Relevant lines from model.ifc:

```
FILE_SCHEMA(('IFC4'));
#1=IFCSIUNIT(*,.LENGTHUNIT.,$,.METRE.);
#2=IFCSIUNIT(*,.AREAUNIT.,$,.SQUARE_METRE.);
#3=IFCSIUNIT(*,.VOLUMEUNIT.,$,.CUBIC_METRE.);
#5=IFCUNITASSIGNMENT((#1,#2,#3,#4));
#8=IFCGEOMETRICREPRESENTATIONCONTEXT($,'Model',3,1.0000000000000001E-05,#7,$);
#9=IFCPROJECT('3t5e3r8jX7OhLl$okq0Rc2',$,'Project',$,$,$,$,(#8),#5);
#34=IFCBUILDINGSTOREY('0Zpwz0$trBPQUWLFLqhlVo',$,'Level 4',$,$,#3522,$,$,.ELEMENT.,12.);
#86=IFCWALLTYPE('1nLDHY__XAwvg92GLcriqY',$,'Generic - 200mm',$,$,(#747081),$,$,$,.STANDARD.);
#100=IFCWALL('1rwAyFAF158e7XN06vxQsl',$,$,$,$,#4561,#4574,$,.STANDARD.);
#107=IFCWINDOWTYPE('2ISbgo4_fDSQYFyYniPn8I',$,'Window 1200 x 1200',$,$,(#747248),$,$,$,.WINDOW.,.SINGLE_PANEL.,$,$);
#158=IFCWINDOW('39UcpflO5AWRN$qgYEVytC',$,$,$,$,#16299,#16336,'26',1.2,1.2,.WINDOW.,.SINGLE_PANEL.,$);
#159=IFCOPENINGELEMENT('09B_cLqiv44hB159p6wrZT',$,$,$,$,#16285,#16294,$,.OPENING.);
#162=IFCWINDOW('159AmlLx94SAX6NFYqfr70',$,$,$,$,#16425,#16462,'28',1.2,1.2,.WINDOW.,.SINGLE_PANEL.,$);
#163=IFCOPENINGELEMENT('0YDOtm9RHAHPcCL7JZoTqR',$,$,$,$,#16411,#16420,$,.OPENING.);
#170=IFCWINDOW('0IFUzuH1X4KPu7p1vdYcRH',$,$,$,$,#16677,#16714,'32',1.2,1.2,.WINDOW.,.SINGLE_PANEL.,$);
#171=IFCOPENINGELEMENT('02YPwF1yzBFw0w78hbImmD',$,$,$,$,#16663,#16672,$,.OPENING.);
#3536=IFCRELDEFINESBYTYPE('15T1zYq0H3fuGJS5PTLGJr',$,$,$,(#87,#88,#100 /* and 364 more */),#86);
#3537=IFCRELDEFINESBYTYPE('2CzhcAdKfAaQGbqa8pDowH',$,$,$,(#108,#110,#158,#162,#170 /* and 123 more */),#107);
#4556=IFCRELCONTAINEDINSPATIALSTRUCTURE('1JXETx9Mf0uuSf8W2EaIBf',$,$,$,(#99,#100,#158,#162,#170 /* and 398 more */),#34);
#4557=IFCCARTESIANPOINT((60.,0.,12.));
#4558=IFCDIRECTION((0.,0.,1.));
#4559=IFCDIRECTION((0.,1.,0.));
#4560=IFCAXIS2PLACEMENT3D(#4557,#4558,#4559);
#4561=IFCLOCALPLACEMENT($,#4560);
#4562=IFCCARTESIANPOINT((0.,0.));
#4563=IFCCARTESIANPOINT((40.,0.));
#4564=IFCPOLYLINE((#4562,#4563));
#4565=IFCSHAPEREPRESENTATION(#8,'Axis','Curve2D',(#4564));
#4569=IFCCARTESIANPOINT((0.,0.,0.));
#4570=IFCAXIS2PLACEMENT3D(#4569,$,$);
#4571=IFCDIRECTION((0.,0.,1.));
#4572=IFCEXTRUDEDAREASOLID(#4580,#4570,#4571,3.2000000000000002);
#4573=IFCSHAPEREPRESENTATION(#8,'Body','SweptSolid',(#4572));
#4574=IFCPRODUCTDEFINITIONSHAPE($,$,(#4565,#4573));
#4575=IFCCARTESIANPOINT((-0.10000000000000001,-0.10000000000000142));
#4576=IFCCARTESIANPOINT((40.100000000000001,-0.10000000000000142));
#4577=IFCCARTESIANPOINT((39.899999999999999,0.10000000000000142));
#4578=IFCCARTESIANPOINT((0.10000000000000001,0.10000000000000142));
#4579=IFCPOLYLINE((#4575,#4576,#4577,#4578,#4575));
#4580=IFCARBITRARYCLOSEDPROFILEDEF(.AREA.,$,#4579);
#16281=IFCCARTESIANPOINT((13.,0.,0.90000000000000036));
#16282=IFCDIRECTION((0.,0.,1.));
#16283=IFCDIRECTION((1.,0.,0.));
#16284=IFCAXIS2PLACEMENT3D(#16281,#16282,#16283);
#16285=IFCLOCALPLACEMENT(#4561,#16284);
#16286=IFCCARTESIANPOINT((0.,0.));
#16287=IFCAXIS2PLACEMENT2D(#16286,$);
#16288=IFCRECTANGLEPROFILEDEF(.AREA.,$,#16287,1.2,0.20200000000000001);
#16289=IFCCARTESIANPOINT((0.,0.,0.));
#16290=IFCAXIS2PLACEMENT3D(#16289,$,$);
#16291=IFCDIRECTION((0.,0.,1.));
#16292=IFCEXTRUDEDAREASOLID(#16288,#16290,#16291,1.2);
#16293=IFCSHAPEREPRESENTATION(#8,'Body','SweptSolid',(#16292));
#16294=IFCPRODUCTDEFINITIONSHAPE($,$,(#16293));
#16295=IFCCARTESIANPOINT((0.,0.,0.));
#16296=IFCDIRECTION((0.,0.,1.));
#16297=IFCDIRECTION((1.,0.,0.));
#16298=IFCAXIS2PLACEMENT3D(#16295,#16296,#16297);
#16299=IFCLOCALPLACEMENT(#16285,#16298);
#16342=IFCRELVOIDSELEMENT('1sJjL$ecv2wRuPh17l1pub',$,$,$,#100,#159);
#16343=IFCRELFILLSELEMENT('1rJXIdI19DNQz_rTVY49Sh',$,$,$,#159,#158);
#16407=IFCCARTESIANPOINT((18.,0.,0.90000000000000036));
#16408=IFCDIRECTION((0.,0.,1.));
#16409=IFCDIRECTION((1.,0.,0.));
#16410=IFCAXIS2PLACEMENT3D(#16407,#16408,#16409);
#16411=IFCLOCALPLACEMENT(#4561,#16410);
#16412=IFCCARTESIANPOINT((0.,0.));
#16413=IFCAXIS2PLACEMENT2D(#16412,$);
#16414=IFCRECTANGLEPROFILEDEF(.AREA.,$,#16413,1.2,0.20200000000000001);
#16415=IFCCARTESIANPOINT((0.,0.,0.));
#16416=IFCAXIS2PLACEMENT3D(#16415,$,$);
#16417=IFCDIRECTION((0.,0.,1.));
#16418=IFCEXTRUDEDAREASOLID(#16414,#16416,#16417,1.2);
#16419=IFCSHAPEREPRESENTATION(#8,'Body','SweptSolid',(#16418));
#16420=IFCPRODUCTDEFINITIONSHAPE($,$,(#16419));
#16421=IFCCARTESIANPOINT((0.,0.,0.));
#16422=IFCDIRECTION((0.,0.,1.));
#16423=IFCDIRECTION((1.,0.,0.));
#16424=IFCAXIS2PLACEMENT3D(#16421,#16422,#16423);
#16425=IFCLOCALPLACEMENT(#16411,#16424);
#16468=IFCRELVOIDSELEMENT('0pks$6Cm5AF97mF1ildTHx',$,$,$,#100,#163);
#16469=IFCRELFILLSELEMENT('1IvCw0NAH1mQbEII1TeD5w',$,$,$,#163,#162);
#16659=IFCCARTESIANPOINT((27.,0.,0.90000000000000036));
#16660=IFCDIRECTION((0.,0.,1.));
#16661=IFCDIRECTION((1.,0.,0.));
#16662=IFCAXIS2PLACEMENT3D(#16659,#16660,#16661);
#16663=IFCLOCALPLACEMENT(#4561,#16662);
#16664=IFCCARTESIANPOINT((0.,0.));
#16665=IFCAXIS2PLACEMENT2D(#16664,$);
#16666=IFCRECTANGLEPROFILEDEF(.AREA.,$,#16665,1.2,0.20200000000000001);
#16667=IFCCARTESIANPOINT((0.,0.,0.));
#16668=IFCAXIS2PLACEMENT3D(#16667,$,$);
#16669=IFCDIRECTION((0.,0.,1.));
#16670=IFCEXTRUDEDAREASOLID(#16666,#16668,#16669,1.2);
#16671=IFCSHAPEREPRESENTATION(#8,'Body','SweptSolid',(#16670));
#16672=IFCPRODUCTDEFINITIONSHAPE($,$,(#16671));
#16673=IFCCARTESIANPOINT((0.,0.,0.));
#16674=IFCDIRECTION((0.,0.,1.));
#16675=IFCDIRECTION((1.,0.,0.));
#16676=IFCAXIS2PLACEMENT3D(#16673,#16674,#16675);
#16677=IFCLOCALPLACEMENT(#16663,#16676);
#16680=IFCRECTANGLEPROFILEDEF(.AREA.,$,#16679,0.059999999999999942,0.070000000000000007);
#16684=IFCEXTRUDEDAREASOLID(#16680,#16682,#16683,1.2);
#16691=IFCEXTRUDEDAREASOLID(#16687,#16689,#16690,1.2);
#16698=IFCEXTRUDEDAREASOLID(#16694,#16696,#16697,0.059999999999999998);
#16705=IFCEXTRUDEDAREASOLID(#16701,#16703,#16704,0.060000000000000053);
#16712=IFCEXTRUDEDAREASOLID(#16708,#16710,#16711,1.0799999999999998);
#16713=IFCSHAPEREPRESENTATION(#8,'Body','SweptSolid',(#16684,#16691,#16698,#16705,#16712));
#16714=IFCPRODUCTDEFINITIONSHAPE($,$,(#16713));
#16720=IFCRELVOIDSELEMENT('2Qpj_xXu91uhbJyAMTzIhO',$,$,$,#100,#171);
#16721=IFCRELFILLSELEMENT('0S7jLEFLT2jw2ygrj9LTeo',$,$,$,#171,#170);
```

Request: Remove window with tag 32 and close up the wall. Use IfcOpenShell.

```python
import ifcopenshell
import ifcopenshell.api.feature
import ifcopenshell.api.root
import ifcopenshell.geom
import ifcopenshell.util.shape

model = ifcopenshell.open("model.ifc")
settings = ifcopenshell.geom.settings()


def volume(element):
    """Net volume in cubic metres, openings subtracted."""
    shape = ifcopenshell.geom.create_shape(settings, element)
    return ifcopenshell.util.shape.get_volume(shape.geometry)


window = model.by_guid("0IFUzuH1X4KPu7p1vdYcRH")
opening = window.FillsVoids[0].RelatingOpeningElement
wall = opening.VoidsElements[0].RelatingBuildingElement
before = volume(wall)

ifcopenshell.api.root.remove_product(model, product=window)
ifcopenshell.api.feature.remove_feature(model, feature=opening)

after = volume(wall)

print(f"wall volume {before:.3f} -> {after:.3f} m3")

model.write("model_updated.ifc")
```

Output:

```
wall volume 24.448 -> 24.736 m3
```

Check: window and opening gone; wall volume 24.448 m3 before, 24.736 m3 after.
